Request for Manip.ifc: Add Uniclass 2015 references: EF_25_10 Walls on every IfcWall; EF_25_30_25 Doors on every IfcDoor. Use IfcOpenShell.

First a look at what the model holds.

```python
import ifcopenshell

model = ifcopenshell.open("Manip.ifc")
print(model.schema)
print("classifications:", [c.Name for c in model.by_type("IfcClassification")])
for ifc_class in ("IfcDoor", "IfcRoof", "IfcStair", "IfcWall", "IfcWindow"):
    print(ifc_class, len(model.by_type(ifc_class)))
```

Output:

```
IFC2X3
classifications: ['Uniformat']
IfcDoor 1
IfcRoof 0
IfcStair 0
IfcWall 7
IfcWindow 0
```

```python
import ifcopenshell
import ifcopenshell.api.classification

model = ifcopenshell.open("Manip.ifc")

# IFC2X3 requires Source and Edition and has no link from the project to the system.
system = model.create_entity("IfcClassification", Source="NBS", Edition="2015", Name="Uniclass 2015")

codes = {
    "IfcWall": ("EF_25_10", "Walls"),
    "IfcDoor": ("EF_25_30_25", "Doors"),
}
for ifc_class, (code, name) in codes.items():
    products = model.by_type(ifc_class)
    ifcopenshell.api.classification.add_reference(
        model, products=products, classification=system, identification=code, name=name
    )
    print(code, len(products))

model.write("Manip-out.ifc")
```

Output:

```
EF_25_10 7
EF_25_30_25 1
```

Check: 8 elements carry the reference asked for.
